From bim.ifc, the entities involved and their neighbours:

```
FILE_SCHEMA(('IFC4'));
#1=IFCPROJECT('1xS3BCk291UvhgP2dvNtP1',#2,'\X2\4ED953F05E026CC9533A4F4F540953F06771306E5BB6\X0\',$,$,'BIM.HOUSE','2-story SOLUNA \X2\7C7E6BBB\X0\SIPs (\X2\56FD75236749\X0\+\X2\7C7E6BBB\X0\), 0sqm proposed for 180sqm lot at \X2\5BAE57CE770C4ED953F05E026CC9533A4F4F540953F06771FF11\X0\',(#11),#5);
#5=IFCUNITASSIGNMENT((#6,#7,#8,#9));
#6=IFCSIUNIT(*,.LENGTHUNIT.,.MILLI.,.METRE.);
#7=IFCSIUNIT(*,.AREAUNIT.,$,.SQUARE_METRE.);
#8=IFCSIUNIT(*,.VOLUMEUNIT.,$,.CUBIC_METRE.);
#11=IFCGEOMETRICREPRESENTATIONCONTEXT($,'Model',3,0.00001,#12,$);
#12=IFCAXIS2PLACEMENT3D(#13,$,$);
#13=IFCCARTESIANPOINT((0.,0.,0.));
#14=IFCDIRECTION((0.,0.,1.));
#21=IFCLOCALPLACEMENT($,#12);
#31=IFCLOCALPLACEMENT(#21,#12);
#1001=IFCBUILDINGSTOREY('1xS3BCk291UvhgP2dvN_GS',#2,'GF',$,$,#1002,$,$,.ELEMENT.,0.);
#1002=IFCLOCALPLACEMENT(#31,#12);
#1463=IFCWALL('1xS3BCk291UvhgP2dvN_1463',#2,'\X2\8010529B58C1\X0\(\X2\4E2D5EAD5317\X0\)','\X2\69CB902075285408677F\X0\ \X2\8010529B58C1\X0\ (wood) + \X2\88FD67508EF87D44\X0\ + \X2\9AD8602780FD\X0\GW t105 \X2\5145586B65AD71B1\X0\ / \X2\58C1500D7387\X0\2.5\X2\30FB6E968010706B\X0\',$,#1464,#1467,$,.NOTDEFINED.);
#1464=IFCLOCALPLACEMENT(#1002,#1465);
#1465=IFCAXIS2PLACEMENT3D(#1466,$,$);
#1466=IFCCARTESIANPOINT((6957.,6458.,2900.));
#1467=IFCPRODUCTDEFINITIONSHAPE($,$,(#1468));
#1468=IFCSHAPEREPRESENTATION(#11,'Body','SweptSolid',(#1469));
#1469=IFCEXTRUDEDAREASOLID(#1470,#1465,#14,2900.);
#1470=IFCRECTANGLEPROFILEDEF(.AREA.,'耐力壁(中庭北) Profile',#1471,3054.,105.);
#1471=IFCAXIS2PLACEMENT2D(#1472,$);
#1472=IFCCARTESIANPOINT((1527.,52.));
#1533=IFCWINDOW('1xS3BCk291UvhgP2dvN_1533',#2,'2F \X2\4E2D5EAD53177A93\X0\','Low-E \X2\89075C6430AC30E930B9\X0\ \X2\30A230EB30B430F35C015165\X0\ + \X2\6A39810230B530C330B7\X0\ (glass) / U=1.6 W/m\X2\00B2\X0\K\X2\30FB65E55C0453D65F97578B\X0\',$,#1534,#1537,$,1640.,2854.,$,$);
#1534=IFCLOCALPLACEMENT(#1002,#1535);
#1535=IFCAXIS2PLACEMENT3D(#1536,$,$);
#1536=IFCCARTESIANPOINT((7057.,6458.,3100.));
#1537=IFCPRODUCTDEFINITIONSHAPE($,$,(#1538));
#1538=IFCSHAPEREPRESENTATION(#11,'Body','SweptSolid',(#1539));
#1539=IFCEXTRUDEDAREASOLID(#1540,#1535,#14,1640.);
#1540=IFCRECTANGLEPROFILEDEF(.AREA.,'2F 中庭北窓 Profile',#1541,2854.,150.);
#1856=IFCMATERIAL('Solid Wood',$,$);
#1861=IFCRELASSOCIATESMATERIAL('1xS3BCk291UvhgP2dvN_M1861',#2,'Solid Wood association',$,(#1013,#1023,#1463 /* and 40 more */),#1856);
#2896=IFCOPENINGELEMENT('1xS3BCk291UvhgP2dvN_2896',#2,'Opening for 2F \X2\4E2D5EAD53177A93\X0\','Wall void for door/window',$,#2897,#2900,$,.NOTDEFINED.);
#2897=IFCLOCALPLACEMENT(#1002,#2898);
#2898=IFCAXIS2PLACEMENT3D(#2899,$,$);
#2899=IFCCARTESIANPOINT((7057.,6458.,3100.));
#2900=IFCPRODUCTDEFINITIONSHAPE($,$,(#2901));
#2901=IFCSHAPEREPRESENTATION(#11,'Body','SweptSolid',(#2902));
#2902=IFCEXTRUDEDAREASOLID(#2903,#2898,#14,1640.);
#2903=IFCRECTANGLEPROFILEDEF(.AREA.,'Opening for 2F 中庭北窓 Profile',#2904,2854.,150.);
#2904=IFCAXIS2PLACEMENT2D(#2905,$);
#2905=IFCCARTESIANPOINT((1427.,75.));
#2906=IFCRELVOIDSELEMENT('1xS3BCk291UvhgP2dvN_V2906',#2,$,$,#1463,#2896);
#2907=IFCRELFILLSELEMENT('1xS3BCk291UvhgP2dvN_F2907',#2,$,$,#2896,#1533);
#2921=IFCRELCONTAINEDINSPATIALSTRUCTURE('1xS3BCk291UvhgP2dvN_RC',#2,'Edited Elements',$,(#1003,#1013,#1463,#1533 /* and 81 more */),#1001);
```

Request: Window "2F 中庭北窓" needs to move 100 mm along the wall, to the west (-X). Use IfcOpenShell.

```python
import ifcopenshell
import ifcopenshell.api.geometry
import ifcopenshell.util.placement

model = ifcopenshell.open("bim.ifc")

window = model.by_guid("1xS3BCk291UvhgP2dvN_1533")
opening = window.FillsVoids[0].RelatingOpeningElement
wall = opening.VoidsElements[0].RelatingBuildingElement

wall_matrix = ifcopenshell.util.placement.get_local_placement(wall.ObjectPlacement)
shift = wall_matrix[:3, 0] * -100.0
before = ifcopenshell.util.placement.get_local_placement(window.ObjectPlacement)[:3, 3].copy()

# The window is not placed relative to its opening, so move both.
for product in (opening, window):
    matrix = ifcopenshell.util.placement.get_local_placement(product.ObjectPlacement)
    matrix[:3, 3] += shift
    ifcopenshell.api.geometry.edit_object_placement(model, product=product, matrix=matrix, is_si=False)

after = ifcopenshell.util.placement.get_local_placement(window.ObjectPlacement)[:3, 3]
print("window moved by", (after - before).round(3) + 0.0)

model.write("bim_rev.ifc")
```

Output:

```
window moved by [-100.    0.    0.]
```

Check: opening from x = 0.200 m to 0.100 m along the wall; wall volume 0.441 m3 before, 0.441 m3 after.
